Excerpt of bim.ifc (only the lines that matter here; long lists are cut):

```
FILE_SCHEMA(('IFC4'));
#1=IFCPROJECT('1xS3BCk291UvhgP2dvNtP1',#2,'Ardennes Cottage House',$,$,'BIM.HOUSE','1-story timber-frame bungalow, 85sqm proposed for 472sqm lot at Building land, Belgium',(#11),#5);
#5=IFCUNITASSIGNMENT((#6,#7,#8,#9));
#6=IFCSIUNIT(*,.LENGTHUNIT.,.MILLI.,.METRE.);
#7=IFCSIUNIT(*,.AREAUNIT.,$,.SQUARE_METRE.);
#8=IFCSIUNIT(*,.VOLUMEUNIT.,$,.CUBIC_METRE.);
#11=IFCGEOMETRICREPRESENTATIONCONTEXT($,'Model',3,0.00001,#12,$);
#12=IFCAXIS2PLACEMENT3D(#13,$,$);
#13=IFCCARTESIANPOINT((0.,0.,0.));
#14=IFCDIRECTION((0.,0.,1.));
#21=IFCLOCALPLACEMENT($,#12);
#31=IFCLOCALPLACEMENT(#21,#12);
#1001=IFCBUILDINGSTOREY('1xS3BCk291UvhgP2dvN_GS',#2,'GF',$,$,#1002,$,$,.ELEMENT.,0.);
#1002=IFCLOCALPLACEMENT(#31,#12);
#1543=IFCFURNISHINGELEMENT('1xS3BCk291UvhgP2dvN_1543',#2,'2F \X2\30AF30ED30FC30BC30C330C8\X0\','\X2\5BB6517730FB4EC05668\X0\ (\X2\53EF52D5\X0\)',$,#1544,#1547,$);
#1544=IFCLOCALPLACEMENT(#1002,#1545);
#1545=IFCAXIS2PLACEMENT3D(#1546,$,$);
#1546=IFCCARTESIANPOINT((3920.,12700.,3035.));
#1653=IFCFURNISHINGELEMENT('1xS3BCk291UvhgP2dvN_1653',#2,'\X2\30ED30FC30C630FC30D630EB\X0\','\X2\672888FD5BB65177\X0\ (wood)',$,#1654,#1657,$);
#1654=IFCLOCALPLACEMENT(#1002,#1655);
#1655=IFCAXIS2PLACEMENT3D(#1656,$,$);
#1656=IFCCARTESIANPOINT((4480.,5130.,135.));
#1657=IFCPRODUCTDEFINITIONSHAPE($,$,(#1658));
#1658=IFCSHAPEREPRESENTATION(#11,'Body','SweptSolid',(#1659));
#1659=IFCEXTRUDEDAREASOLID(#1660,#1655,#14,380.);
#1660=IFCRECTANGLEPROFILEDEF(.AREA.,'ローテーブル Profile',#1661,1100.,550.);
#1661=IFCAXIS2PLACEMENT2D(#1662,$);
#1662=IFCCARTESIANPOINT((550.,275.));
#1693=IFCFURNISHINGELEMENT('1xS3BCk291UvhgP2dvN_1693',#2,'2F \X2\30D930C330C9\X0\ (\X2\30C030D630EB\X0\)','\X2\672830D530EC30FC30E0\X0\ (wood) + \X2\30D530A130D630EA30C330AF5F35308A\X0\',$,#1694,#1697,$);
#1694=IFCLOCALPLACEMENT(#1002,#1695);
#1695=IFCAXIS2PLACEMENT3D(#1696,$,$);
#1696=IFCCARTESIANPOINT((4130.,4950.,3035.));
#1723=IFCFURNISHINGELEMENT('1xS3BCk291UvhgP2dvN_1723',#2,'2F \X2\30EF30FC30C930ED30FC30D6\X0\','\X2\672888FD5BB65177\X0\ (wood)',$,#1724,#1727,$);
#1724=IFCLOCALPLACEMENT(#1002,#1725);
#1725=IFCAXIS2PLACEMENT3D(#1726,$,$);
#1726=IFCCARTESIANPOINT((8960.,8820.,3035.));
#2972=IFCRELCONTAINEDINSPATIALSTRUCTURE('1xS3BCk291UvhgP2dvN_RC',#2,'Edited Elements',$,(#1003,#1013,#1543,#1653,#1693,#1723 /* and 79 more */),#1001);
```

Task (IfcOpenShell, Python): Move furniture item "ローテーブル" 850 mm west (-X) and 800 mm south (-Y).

```python
import ifcopenshell
import ifcopenshell.api.geometry
import ifcopenshell.util.placement

model = ifcopenshell.open("bim.ifc")

item = model.by_guid("1xS3BCk291UvhgP2dvN_1653")
matrix = ifcopenshell.util.placement.get_local_placement(item.ObjectPlacement)
matrix[0, 3] -= 850.0
matrix[1, 3] -= 800.0
ifcopenshell.api.geometry.edit_object_placement(model, product=item, matrix=matrix, is_si=False)

print(ifcopenshell.util.placement.get_local_placement(item.ObjectPlacement).round(3) + 0.0)

model.write("bim_v2.ifc")
```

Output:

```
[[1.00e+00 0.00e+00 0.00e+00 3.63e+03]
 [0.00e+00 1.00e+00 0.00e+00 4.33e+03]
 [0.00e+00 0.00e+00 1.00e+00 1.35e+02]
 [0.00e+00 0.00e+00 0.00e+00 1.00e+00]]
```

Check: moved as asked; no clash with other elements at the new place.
